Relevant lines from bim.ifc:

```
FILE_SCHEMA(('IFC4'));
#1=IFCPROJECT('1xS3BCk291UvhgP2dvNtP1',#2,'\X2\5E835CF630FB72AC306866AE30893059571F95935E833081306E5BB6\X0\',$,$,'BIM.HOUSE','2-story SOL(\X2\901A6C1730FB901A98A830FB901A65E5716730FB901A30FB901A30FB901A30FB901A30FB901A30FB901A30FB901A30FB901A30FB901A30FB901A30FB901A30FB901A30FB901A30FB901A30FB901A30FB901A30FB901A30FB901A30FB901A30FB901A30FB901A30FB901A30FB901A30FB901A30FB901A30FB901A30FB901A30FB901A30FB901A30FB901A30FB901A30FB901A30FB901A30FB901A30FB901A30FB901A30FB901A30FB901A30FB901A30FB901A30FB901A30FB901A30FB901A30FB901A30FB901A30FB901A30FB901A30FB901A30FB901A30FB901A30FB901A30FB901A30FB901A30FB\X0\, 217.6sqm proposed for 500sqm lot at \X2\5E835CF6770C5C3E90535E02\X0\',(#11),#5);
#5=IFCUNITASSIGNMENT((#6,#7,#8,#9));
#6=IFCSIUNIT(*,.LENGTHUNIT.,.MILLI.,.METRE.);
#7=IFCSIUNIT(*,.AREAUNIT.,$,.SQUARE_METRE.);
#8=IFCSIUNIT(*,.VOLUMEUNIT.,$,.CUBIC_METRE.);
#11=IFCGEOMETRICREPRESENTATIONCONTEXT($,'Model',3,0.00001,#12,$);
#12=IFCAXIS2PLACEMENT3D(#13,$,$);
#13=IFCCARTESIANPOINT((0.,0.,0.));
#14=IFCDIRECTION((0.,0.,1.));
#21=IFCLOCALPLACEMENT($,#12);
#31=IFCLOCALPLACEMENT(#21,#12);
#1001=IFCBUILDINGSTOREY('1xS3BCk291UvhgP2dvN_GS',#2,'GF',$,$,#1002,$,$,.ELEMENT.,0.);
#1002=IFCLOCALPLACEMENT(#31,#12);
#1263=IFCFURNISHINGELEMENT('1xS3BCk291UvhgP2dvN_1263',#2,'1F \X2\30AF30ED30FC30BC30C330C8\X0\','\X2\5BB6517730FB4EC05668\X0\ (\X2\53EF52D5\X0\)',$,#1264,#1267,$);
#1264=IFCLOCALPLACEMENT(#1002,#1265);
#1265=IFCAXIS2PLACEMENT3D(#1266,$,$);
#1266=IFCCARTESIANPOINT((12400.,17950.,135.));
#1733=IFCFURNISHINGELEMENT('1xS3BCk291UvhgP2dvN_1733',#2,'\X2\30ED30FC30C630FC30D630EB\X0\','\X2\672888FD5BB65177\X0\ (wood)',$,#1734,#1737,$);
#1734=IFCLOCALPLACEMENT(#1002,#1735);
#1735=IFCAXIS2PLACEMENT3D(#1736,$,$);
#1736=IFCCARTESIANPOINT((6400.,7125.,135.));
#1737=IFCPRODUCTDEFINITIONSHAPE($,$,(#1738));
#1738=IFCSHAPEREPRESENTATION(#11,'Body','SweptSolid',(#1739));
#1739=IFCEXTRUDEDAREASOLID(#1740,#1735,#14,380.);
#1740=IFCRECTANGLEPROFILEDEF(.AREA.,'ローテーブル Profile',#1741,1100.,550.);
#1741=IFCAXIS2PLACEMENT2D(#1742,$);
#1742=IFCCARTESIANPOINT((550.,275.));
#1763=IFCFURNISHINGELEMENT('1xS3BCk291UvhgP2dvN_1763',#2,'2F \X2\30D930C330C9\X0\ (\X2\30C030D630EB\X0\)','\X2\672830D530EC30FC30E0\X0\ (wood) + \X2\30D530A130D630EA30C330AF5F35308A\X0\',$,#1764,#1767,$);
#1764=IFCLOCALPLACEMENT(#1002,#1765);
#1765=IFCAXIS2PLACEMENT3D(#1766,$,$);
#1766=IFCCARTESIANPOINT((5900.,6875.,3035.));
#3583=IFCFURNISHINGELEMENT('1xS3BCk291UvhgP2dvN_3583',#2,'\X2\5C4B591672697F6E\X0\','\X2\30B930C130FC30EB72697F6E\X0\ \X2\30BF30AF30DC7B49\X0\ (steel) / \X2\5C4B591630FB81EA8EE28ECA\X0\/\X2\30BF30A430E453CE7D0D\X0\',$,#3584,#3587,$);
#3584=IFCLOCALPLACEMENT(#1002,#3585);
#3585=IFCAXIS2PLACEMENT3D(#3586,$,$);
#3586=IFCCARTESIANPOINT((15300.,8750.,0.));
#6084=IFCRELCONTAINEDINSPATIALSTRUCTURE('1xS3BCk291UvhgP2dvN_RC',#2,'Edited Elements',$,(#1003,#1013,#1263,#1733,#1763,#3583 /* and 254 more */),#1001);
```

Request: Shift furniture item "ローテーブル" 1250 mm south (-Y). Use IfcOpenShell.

```python
import ifcopenshell
import ifcopenshell.api.geometry
import ifcopenshell.util.placement
import ifcopenshell.util.unit

model = ifcopenshell.open("bim.ifc")
unit_scale = ifcopenshell.util.unit.calculate_unit_scale(model)

item = model.by_id(1733)
matrix = ifcopenshell.util.placement.get_local_placement(item.ObjectPlacement)
matrix[1, 3] -= 1.25 / unit_scale
ifcopenshell.api.geometry.edit_object_placement(model, product=item, matrix=matrix, is_si=False)

print(ifcopenshell.util.placement.get_local_placement(item.ObjectPlacement).round(3) + 0.0)

model.write("bim_updated.ifc")
```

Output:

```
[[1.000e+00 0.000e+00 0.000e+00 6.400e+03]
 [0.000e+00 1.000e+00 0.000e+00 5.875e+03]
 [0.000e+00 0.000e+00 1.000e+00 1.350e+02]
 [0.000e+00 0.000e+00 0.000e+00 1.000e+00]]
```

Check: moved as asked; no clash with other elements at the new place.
